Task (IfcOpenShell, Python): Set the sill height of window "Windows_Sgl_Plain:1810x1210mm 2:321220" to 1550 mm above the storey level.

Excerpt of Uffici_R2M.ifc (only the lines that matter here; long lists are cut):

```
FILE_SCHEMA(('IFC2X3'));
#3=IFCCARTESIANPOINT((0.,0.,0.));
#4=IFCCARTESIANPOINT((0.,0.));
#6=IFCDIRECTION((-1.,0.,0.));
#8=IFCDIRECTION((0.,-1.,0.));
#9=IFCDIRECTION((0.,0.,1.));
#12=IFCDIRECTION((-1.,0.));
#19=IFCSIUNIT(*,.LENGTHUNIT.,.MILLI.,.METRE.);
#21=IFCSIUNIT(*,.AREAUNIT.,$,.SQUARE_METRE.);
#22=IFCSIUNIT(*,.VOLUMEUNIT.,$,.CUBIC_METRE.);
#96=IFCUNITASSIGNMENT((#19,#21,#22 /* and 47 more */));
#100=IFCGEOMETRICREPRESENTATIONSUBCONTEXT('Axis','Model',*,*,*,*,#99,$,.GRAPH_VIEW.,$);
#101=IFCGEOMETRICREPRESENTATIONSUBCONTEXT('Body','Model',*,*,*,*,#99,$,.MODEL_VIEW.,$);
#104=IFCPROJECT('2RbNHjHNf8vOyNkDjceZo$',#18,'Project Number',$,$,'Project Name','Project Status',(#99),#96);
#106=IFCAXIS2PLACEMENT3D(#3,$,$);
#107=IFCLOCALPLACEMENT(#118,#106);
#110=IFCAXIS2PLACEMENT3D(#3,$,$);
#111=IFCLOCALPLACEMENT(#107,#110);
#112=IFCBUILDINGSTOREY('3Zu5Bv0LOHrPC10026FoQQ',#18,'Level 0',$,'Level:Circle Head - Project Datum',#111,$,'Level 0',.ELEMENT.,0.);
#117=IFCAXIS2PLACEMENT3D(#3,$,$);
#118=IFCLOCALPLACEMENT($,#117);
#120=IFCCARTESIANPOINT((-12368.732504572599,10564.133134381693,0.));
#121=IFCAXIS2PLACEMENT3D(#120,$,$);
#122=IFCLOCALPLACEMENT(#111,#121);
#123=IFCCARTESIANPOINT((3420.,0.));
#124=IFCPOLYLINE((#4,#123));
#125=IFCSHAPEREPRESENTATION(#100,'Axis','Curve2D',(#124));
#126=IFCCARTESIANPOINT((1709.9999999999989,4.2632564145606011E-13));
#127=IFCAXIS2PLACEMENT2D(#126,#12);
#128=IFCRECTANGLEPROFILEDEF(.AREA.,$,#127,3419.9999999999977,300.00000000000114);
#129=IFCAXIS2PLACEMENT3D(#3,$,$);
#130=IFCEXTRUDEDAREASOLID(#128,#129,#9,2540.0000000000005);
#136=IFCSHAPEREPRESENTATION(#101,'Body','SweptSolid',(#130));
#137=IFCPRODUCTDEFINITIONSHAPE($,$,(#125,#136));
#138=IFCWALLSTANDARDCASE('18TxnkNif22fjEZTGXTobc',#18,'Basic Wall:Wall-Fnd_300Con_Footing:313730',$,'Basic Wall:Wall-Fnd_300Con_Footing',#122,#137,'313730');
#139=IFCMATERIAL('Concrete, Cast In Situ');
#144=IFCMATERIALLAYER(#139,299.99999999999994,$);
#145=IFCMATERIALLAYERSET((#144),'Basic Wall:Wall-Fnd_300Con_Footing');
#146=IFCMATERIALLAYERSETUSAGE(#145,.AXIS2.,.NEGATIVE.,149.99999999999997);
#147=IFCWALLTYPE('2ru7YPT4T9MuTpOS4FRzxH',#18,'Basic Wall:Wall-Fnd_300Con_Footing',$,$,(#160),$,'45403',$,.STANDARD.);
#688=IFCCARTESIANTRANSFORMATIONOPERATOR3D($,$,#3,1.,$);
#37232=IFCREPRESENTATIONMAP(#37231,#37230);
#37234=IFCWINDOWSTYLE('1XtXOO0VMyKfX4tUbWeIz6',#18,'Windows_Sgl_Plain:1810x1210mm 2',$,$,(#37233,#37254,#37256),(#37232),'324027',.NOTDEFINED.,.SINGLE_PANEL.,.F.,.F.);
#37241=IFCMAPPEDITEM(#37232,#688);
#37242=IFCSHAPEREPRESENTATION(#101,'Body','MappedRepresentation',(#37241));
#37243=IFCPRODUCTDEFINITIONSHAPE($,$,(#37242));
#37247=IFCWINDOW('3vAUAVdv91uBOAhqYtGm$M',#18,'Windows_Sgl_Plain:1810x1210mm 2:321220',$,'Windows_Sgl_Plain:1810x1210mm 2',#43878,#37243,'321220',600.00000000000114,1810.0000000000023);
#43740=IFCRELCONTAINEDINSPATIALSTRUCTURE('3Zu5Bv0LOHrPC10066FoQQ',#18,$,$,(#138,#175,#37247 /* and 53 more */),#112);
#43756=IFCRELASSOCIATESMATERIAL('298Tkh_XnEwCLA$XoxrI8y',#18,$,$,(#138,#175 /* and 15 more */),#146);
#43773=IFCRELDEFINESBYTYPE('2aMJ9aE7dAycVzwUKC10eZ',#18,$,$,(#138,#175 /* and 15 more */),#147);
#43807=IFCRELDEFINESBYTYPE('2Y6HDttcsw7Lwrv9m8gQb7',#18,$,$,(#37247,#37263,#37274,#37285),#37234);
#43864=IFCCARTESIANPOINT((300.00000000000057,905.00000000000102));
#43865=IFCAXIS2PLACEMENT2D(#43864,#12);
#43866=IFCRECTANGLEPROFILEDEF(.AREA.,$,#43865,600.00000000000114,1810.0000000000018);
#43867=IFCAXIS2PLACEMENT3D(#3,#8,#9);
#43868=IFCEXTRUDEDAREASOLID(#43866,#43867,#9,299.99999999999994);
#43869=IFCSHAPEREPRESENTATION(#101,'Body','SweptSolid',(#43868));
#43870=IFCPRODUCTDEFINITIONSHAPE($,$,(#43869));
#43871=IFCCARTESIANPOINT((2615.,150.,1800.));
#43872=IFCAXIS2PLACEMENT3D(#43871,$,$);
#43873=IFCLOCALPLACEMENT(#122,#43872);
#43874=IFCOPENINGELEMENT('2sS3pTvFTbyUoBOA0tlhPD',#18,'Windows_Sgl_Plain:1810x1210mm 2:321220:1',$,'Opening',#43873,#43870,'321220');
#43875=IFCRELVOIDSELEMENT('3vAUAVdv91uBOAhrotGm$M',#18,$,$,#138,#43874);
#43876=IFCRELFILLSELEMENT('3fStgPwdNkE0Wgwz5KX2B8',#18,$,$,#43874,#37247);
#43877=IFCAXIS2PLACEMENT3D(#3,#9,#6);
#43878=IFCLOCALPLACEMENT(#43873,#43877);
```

```python
import numpy as np
import ifcopenshell
import ifcopenshell.api.geometry
import ifcopenshell.geom
import ifcopenshell.util.element
import ifcopenshell.util.placement
import ifcopenshell.util.shape
import ifcopenshell.util.unit

model = ifcopenshell.open("Uffici_R2M.ifc")
unit_scale = ifcopenshell.util.unit.calculate_unit_scale(model)

window = model.by_guid("3vAUAVdv91uBOAhqYtGm$M")
opening = window.FillsVoids[0].RelatingOpeningElement
storey = ifcopenshell.util.element.get_container(window, ifc_class="IfcBuildingStorey")
level = ifcopenshell.util.placement.get_local_placement(storey.ObjectPlacement)[2, 3]

# The opening's origin need not be at the sill, so measure its lowest point.
shape = ifcopenshell.geom.create_shape(ifcopenshell.geom.settings(), opening)
bottom = ifcopenshell.util.shape.get_shape_bottom_elevation(shape, shape.geometry) / unit_scale
dz = level + 1.55 / unit_scale - bottom

shift = np.array([0.0, 0.0, dz])
# The window is placed relative to its opening, so it follows when the opening moves.
matrix = ifcopenshell.util.placement.get_local_placement(opening.ObjectPlacement)
matrix[:3, 3] += shift
ifcopenshell.api.geometry.edit_object_placement(
    model, product=opening, matrix=matrix, is_si=False, should_transform_children=True
)

print(f"moved by {dz * unit_scale:+.3f} m")

model.write("Uffici_R2M_v2.ifc")
```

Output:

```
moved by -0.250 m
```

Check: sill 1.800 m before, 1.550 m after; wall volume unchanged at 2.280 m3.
